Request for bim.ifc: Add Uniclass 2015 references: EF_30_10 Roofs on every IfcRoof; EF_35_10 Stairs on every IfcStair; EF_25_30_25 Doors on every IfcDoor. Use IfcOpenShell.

First a look at what the model holds.

```python
import ifcopenshell

model = ifcopenshell.open("bim.ifc")
print(model.schema)
print("classifications:", [c.Name for c in model.by_type("IfcClassification")])
for ifc_class in ("IfcDoor", "IfcRoof", "IfcStair", "IfcWall", "IfcWindow"):
    print(ifc_class, len(model.by_type(ifc_class)))
```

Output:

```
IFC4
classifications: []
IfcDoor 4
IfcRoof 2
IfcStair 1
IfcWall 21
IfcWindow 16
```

```python
import ifcopenshell
import ifcopenshell.api.classification

model = ifcopenshell.open("bim.ifc")

system = ifcopenshell.api.classification.add_classification(model, classification="Uniclass 2015")

codes = {
    "IfcRoof": ("EF_30_10", "Roofs"),
    "IfcStair": ("EF_35_10", "Stairs"),
    "IfcDoor": ("EF_25_30_25", "Doors"),
}
for ifc_class, (code, name) in codes.items():
    products = model.by_type(ifc_class)
    ifcopenshell.api.classification.add_reference(
        model, products=products, classification=system, identification=code, name=name
    )
    print(code, len(products))

model.write("bim_v2.ifc")
```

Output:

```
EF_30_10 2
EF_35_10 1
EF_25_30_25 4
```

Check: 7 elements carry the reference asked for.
